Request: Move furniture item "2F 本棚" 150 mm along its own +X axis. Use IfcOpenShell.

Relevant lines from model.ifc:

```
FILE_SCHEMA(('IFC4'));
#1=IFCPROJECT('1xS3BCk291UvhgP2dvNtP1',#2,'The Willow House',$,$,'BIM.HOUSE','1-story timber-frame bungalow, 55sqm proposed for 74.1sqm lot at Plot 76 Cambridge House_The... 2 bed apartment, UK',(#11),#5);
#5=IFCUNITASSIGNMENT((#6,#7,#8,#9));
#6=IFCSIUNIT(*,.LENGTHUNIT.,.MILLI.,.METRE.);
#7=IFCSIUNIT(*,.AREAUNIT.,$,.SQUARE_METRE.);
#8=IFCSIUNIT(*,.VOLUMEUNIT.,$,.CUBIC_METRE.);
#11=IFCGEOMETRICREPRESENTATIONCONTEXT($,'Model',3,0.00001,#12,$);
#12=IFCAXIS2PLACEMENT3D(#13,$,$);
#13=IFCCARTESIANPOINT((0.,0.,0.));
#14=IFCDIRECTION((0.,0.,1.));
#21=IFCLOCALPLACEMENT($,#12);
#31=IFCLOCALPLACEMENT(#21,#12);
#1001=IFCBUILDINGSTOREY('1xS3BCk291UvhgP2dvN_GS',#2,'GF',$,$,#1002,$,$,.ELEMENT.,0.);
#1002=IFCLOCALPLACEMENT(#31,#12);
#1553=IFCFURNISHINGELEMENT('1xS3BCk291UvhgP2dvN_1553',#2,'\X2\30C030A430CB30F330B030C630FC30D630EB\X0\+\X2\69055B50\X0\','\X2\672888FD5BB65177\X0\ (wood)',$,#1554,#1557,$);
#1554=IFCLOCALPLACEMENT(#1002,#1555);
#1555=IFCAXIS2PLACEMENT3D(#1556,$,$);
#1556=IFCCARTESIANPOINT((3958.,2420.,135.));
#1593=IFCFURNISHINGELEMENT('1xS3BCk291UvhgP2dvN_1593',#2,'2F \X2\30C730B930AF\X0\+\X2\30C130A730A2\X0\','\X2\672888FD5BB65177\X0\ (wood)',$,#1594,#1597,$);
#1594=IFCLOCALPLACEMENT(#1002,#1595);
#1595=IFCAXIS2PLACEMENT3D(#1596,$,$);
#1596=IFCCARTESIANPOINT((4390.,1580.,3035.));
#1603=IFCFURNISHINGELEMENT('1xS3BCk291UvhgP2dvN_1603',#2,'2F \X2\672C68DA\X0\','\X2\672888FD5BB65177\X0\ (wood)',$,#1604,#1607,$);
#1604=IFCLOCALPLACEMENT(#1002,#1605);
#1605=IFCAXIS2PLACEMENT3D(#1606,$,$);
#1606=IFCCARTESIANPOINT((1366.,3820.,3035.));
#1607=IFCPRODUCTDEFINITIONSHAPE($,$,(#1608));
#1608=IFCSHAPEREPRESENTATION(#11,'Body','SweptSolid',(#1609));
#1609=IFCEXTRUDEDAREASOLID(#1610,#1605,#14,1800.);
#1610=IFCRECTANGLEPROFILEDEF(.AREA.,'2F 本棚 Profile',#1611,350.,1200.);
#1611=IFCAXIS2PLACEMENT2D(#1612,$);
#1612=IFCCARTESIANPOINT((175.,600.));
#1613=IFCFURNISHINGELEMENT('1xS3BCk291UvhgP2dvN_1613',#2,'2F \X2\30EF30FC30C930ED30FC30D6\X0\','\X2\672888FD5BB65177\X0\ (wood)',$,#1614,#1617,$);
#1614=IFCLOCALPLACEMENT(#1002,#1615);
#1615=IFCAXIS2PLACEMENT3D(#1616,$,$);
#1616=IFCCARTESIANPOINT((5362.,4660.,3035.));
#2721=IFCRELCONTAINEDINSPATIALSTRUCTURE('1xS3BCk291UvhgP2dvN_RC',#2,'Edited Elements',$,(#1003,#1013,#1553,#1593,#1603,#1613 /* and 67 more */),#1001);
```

```python
import ifcopenshell
import ifcopenshell.api.geometry
import ifcopenshell.util.placement
import ifcopenshell.util.unit

model = ifcopenshell.open("model.ifc")
unit_scale = ifcopenshell.util.unit.calculate_unit_scale(model)

item = model.by_guid("1xS3BCk291UvhgP2dvN_1603")
matrix = ifcopenshell.util.placement.get_local_placement(item.ObjectPlacement)
matrix[:3, 3] += matrix[:3, 0] * 0.15 / unit_scale
ifcopenshell.api.geometry.edit_object_placement(model, product=item, matrix=matrix, is_si=False)

print(ifcopenshell.util.placement.get_local_placement(item.ObjectPlacement).round(3) + 0.0)

model.write("model_edited.ifc")
```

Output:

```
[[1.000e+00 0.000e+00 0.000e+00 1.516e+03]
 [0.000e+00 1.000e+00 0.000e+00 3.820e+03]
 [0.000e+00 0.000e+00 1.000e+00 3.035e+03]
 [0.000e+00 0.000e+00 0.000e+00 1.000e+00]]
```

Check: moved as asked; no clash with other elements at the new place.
